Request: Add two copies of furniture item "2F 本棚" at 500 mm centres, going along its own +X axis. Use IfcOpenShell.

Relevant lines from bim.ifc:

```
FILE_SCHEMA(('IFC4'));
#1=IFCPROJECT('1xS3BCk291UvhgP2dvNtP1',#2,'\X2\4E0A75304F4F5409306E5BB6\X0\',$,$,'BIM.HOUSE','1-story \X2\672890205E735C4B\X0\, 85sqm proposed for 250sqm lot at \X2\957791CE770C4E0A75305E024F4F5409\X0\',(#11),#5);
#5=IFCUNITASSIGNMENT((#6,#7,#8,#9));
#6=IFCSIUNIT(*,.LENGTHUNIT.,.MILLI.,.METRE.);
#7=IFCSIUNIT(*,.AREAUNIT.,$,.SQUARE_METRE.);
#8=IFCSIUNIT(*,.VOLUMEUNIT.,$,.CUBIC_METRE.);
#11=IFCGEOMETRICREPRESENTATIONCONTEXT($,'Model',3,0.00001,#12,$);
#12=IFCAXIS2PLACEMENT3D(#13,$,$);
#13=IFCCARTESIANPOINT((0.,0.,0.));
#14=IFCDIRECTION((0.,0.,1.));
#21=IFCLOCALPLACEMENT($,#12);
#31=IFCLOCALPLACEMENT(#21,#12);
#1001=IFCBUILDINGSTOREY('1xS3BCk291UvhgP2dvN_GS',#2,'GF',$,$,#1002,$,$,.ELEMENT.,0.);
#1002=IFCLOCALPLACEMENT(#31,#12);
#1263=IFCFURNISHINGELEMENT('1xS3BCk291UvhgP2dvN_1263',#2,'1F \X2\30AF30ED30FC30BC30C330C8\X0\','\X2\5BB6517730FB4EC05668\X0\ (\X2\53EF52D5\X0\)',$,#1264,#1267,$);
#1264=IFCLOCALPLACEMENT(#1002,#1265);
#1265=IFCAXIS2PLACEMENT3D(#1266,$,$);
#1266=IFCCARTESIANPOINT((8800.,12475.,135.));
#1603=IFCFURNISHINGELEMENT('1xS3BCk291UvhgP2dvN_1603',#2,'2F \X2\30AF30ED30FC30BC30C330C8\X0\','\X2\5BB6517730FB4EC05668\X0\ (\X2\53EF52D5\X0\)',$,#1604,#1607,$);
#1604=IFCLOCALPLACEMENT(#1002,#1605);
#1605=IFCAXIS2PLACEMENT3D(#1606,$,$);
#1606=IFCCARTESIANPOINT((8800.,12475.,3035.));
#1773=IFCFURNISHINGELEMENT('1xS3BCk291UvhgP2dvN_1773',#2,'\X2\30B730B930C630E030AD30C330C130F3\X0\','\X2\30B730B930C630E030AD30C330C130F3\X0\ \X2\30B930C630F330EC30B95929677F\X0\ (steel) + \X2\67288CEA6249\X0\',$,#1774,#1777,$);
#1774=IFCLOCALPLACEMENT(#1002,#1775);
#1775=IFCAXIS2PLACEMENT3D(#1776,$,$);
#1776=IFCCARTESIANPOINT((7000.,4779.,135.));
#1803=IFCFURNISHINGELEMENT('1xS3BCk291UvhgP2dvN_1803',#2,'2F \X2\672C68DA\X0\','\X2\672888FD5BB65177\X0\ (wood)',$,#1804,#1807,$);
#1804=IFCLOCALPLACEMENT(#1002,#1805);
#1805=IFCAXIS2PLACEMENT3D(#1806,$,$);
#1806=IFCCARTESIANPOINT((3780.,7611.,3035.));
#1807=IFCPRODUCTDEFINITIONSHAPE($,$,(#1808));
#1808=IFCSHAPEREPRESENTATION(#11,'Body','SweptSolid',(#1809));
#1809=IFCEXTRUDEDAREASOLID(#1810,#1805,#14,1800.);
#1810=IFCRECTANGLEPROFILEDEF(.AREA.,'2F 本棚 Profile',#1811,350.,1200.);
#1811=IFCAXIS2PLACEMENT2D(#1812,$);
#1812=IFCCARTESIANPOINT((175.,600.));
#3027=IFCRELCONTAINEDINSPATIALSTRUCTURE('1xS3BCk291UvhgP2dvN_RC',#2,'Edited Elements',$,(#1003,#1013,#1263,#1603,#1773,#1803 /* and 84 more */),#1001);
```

```python
import ifcopenshell
import ifcopenshell.api.geometry
import ifcopenshell.api.root
import ifcopenshell.util.element
import ifcopenshell.util.placement
import ifcopenshell.util.unit

model = ifcopenshell.open("bim.ifc")
unit_scale = ifcopenshell.util.unit.calculate_unit_scale(model)


def reuse_history(source, copy):
    """copy_class also copies each property set's owner history, people and application; keep the originals."""
    for rel in copy.IsDefinedBy:
        if rel.is_a("IfcRelDefinesByProperties") and (history := rel.RelatingPropertyDefinition.OwnerHistory):
            rel.RelatingPropertyDefinition.OwnerHistory = source.OwnerHistory
            ifcopenshell.util.element.remove_deep2(model, history)


source = model.by_guid("1xS3BCk291UvhgP2dvN_1803")
base = ifcopenshell.util.placement.get_local_placement(source.ObjectPlacement)
step = base[:3, 0] * 0.5 / unit_scale

for i in range(1, 3):
    copy = ifcopenshell.api.root.copy_class(model, product=source)
    copy.Representation = ifcopenshell.util.element.copy_deep(
        model, source.Representation, exclude=["IfcGeometricRepresentationContext", "IfcRepresentationMap"]
    )
    reuse_history(source, copy)
    matrix = base.copy()
    matrix[:3, 3] += i * step
    print("added at", matrix[:3, 3].round(3) + 0.0)
    ifcopenshell.api.geometry.edit_object_placement(model, product=copy, matrix=matrix, is_si=False)

model.write("bim_v2.ifc")
```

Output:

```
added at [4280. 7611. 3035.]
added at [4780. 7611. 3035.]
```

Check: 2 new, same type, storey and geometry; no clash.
